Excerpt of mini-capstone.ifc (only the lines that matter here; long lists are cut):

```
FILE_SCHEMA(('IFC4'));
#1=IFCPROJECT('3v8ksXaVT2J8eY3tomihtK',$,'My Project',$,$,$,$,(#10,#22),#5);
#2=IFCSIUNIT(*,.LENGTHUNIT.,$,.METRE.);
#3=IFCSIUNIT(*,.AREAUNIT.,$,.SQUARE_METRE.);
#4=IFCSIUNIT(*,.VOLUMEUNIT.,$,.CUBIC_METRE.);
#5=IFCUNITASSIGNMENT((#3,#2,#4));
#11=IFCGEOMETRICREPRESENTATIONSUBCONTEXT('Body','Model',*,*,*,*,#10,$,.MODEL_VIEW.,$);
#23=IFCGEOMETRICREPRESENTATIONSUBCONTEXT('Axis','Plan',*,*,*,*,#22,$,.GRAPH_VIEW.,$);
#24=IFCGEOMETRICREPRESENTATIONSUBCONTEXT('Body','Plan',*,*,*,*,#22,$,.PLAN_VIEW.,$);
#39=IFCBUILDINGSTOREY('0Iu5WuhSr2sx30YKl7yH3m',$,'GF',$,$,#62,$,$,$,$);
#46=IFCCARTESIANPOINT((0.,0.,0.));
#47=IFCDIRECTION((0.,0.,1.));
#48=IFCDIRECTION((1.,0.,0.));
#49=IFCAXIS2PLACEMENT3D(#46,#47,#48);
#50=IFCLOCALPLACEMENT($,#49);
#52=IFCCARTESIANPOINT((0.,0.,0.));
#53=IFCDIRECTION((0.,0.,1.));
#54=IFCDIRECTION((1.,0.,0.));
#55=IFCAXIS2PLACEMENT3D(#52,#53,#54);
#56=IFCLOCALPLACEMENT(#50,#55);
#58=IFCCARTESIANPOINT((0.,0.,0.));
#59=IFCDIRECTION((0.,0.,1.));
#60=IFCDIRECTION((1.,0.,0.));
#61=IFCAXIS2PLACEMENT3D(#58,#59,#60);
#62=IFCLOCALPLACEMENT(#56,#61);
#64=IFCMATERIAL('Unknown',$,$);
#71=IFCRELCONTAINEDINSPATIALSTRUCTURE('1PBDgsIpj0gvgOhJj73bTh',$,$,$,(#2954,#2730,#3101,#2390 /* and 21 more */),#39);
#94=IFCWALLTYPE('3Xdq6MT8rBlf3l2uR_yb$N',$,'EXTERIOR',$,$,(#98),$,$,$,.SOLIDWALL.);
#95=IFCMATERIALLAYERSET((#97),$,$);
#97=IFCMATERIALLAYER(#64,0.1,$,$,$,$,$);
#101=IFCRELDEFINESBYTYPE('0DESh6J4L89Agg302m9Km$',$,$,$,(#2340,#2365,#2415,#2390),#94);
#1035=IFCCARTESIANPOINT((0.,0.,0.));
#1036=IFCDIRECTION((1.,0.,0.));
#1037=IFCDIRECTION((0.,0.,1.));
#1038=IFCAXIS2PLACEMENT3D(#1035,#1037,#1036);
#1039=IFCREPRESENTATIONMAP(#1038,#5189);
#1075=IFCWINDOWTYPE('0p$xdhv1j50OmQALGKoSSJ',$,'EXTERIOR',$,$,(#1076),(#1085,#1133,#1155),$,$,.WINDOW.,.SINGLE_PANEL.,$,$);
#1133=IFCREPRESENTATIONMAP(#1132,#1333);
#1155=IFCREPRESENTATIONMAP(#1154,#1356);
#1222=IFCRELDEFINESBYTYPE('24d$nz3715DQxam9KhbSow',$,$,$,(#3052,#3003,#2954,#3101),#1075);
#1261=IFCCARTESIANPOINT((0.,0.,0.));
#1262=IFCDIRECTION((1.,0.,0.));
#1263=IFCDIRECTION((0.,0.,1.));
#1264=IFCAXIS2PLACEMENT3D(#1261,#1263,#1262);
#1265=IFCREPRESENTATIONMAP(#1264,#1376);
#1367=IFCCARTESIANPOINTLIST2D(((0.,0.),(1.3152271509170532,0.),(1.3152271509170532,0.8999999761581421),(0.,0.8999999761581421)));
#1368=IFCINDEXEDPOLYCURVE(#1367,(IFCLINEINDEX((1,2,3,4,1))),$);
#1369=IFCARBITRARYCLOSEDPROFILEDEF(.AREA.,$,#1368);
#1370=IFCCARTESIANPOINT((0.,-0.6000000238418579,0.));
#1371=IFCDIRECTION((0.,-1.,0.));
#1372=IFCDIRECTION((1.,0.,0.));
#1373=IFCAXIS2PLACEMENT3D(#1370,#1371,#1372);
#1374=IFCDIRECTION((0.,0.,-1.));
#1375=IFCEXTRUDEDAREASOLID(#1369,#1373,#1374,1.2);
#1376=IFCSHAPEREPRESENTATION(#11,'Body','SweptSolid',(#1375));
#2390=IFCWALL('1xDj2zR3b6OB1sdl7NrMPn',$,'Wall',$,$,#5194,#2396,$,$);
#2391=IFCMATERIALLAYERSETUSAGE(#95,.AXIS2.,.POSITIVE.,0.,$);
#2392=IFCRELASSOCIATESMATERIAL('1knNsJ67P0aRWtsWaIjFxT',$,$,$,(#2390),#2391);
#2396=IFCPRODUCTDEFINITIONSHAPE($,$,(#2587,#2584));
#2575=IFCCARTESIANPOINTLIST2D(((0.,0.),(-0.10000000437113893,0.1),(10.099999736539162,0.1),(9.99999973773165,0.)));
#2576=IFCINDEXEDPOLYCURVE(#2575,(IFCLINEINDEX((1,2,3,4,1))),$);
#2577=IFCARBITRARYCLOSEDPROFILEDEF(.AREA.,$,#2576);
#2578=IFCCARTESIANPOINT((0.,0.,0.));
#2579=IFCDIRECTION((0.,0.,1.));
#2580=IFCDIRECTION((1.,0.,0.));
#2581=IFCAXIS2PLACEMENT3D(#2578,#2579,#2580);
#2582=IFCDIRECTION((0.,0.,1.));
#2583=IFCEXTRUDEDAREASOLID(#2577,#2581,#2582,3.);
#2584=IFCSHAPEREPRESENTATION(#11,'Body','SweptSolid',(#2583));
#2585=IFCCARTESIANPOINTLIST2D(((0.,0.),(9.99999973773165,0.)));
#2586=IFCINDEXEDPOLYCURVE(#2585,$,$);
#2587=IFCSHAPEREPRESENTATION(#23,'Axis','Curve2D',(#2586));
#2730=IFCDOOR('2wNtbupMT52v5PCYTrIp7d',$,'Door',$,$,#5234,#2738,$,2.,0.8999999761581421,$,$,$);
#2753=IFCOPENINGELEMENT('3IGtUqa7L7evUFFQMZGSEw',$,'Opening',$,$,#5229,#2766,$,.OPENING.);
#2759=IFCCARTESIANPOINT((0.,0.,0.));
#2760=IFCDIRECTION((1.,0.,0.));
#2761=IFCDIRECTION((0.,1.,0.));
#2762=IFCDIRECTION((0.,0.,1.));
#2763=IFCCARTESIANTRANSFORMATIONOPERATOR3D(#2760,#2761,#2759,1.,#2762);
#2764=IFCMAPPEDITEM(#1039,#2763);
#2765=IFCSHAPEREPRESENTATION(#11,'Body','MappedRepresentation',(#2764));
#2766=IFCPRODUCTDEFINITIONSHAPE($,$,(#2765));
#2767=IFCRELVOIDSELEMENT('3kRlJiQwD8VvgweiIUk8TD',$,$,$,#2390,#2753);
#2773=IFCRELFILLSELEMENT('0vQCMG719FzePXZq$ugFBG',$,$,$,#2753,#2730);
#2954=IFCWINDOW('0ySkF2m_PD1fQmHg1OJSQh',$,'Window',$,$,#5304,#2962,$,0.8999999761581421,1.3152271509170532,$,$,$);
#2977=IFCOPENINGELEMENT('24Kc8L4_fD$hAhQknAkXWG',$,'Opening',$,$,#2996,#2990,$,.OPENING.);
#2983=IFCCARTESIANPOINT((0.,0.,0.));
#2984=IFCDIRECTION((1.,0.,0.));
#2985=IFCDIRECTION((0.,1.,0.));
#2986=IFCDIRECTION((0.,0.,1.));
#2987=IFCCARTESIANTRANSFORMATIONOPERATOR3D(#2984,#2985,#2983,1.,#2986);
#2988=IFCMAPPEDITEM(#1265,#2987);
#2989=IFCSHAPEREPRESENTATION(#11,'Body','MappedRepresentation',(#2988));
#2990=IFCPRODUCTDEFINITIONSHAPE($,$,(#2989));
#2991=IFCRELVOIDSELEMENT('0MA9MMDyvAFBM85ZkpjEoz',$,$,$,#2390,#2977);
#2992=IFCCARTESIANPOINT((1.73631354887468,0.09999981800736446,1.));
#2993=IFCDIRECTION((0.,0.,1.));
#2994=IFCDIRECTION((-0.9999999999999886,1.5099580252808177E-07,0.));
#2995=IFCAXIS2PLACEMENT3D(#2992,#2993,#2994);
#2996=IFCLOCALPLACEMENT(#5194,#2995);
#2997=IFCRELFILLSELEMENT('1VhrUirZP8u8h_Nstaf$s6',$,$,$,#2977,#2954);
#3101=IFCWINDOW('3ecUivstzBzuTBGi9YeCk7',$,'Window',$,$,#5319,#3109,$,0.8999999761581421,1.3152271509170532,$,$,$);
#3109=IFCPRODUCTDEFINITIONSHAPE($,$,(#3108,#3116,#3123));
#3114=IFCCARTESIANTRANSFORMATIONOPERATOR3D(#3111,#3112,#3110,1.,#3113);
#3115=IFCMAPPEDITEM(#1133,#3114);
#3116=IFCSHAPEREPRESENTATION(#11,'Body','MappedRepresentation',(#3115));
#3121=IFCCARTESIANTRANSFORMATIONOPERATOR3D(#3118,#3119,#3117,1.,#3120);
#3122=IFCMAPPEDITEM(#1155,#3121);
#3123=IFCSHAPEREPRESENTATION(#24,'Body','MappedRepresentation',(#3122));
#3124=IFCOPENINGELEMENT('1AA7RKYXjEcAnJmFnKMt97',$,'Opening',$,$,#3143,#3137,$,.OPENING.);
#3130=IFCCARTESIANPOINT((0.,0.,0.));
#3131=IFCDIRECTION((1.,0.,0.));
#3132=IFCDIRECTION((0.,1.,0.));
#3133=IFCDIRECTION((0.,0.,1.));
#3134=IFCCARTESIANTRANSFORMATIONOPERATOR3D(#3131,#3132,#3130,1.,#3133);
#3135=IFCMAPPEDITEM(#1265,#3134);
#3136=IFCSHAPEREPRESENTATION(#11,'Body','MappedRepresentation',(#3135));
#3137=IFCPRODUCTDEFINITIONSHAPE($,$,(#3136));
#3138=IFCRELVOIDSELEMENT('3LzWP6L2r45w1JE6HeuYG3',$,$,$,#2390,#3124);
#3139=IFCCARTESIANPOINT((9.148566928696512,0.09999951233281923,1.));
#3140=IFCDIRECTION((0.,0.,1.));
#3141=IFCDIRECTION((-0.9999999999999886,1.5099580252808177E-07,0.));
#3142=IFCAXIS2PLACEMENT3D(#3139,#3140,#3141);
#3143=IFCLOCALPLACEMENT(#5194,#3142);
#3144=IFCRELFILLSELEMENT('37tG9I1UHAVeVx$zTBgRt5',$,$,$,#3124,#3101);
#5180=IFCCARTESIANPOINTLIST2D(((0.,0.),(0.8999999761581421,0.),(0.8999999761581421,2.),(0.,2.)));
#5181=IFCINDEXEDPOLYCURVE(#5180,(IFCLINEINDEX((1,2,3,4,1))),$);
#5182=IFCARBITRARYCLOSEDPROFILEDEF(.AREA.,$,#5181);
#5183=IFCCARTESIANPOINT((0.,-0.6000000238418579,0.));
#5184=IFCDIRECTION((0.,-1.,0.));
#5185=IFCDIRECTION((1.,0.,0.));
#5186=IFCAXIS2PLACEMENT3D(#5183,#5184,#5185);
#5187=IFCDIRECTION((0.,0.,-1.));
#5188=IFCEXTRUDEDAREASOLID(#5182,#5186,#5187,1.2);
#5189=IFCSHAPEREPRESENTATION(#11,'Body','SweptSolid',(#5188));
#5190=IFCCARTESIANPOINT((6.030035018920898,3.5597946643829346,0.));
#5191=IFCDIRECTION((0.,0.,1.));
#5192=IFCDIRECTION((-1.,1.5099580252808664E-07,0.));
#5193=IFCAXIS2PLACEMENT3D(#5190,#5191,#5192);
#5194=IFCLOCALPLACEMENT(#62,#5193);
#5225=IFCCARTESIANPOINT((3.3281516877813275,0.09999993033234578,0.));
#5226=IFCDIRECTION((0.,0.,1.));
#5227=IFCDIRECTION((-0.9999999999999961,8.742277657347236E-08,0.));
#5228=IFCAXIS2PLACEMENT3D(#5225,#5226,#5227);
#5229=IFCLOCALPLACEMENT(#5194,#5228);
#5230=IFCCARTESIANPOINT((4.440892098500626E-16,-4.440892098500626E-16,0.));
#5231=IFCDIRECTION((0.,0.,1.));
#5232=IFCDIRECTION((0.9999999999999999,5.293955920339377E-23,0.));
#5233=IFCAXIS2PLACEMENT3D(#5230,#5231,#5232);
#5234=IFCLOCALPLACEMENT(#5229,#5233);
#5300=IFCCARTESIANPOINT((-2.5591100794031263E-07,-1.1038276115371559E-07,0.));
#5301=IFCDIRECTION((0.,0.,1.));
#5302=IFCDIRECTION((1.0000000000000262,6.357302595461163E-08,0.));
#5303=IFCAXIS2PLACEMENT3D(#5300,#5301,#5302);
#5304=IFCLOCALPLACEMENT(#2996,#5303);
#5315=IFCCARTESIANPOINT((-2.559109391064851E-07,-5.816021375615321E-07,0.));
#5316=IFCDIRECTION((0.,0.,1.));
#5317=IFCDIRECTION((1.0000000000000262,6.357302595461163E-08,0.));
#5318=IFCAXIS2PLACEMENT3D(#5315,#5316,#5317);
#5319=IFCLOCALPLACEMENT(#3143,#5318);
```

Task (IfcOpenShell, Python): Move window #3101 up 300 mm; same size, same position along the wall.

```python
import numpy as np
import ifcopenshell
import ifcopenshell.api.geometry
import ifcopenshell.util.placement
import ifcopenshell.util.unit

model = ifcopenshell.open("mini-capstone.ifc")
unit_scale = ifcopenshell.util.unit.calculate_unit_scale(model)

window = model.by_id(3101)
opening = window.FillsVoids[0].RelatingOpeningElement
dz = 0.3 / unit_scale

shift = np.array([0.0, 0.0, dz])
# The window is placed relative to its opening, so it follows when the opening moves.
matrix = ifcopenshell.util.placement.get_local_placement(opening.ObjectPlacement)
matrix[:3, 3] += shift
ifcopenshell.api.geometry.edit_object_placement(
    model, product=opening, matrix=matrix, is_si=False, should_transform_children=True
)

print(f"moved by {dz * unit_scale:+.3f} m")

model.write("mini-capstone-out.ifc")
```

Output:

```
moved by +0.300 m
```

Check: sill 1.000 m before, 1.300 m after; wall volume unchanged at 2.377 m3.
